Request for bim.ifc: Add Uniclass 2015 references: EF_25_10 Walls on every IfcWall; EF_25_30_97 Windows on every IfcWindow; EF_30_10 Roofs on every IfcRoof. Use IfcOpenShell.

First a look at what the model holds.

```python
import ifcopenshell

model = ifcopenshell.open("bim.ifc")
print(model.schema)
print("classifications:", [c.Name for c in model.by_type("IfcClassification")])
for ifc_class in ("IfcDoor", "IfcRoof", "IfcStair", "IfcWall", "IfcWindow"):
    print(ifc_class, len(model.by_type(ifc_class)))
```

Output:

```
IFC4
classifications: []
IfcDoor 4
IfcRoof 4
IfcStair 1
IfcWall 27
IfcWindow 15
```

```python
import ifcopenshell
import ifcopenshell.api.classification

model = ifcopenshell.open("bim.ifc")

system = ifcopenshell.api.classification.add_classification(model, classification="Uniclass 2015")

codes = {
    "IfcWall": ("EF_25_10", "Walls"),
    "IfcWindow": ("EF_25_30_97", "Windows"),
    "IfcRoof": ("EF_30_10", "Roofs"),
}
for ifc_class, (code, name) in codes.items():
    products = model.by_type(ifc_class)
    ifcopenshell.api.classification.add_reference(
        model, products=products, classification=system, identification=code, name=name
    )
    print(code, len(products))

model.write("bim-out.ifc")
```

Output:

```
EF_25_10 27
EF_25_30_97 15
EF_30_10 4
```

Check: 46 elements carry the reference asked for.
